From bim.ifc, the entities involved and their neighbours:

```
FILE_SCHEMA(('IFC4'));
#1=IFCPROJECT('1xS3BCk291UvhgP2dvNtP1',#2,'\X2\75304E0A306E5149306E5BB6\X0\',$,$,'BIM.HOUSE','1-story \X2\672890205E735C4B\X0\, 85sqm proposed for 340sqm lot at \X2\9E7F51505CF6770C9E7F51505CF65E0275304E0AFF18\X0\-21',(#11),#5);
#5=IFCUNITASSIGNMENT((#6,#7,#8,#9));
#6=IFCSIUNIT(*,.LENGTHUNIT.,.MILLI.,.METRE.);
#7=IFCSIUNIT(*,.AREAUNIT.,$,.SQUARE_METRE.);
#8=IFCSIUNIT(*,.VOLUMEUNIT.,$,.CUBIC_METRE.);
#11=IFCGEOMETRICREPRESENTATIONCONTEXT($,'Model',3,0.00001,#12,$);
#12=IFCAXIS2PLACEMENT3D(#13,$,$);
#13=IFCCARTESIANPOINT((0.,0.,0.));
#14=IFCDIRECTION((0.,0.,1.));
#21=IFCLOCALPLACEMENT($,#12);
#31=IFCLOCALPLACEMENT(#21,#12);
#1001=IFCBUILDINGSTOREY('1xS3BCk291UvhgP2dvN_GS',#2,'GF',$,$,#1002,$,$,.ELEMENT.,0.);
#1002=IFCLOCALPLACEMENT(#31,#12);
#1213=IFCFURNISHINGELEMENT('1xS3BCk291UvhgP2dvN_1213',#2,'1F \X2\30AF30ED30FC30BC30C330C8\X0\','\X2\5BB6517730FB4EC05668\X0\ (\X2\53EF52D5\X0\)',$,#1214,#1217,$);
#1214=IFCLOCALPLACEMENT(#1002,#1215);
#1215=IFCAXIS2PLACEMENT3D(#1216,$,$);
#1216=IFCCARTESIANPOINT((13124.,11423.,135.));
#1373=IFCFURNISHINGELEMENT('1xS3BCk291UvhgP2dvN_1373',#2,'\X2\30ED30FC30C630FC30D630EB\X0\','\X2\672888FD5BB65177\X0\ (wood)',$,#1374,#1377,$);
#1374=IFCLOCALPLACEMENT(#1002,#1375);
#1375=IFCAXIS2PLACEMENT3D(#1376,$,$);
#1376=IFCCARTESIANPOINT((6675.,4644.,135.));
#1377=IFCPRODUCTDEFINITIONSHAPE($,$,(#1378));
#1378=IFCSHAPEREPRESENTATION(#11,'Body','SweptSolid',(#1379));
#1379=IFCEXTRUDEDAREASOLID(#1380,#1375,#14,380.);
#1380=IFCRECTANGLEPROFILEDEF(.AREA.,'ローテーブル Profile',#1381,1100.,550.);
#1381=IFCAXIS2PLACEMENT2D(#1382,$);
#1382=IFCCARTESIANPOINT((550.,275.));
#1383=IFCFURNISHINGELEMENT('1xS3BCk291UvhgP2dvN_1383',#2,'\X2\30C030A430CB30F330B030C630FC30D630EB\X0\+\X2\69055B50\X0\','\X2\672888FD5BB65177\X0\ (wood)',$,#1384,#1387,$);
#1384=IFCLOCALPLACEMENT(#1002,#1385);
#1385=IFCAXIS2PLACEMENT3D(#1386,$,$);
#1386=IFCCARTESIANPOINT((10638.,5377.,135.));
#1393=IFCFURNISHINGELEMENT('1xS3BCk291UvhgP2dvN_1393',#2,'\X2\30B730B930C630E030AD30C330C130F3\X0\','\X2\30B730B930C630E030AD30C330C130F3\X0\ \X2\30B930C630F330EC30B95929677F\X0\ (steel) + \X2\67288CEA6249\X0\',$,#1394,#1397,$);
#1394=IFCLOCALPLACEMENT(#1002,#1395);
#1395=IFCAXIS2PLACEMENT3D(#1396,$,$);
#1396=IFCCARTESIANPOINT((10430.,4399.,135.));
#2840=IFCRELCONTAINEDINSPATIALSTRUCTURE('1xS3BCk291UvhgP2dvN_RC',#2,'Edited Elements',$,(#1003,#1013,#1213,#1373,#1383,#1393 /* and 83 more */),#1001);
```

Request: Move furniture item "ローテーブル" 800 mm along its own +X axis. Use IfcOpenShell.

```python
import ifcopenshell
import ifcopenshell.api.geometry
import ifcopenshell.util.placement
import ifcopenshell.util.unit

model = ifcopenshell.open("bim.ifc")
unit_scale = ifcopenshell.util.unit.calculate_unit_scale(model)

item = model.by_guid("1xS3BCk291UvhgP2dvN_1373")
matrix = ifcopenshell.util.placement.get_local_placement(item.ObjectPlacement)
matrix[:3, 3] += matrix[:3, 0] * 0.8 / unit_scale
ifcopenshell.api.geometry.edit_object_placement(model, product=item, matrix=matrix, is_si=False)

print(ifcopenshell.util.placement.get_local_placement(item.ObjectPlacement).round(3) + 0.0)

model.write("bim_updated.ifc")
```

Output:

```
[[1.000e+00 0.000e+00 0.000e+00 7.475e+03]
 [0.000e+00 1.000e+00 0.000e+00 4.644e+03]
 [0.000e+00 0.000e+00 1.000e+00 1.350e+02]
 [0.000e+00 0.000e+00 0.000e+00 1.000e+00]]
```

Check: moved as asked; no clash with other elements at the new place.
